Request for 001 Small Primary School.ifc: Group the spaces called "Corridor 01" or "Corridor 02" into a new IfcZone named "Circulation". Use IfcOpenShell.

First a look at what the model holds.

```python
import ifcopenshell

model = ifcopenshell.open("001 Small Primary School.ifc")
print(model.schema)
seen = {}
for space in model.by_type("IfcSpace"):
    seen[space.LongName] = seen.get(space.LongName, 0) + 1
for name, count in sorted(seen.items(), key=str):
    print(count, "x", name)
print("zones:", [z.Name for z in model.by_type("IfcZone")][:20])
```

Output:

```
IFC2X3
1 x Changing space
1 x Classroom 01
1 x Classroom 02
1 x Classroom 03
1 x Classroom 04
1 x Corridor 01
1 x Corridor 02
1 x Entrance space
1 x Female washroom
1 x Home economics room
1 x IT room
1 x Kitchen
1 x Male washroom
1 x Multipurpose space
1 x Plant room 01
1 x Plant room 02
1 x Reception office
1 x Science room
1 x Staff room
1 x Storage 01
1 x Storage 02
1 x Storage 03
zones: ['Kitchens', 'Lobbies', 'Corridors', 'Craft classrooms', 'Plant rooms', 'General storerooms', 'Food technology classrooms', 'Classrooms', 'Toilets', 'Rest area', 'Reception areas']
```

```python
import ifcopenshell
import ifcopenshell.api.group
import ifcopenshell.api.root

model = ifcopenshell.open("001 Small Primary School.ifc")

names = {"Corridor 01", "Corridor 02"}
spaces = [s for s in model.by_type("IfcSpace") if s.LongName in names]

zone = ifcopenshell.api.root.create_entity(model, ifc_class="IfcZone", name="Circulation")
ifcopenshell.api.group.assign_group(model, products=spaces, group=zone)
print(len(spaces), "spaces in", zone.Name)

model.write("001 Small Primary School_v2.ifc")
```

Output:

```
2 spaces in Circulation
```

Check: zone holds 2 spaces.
